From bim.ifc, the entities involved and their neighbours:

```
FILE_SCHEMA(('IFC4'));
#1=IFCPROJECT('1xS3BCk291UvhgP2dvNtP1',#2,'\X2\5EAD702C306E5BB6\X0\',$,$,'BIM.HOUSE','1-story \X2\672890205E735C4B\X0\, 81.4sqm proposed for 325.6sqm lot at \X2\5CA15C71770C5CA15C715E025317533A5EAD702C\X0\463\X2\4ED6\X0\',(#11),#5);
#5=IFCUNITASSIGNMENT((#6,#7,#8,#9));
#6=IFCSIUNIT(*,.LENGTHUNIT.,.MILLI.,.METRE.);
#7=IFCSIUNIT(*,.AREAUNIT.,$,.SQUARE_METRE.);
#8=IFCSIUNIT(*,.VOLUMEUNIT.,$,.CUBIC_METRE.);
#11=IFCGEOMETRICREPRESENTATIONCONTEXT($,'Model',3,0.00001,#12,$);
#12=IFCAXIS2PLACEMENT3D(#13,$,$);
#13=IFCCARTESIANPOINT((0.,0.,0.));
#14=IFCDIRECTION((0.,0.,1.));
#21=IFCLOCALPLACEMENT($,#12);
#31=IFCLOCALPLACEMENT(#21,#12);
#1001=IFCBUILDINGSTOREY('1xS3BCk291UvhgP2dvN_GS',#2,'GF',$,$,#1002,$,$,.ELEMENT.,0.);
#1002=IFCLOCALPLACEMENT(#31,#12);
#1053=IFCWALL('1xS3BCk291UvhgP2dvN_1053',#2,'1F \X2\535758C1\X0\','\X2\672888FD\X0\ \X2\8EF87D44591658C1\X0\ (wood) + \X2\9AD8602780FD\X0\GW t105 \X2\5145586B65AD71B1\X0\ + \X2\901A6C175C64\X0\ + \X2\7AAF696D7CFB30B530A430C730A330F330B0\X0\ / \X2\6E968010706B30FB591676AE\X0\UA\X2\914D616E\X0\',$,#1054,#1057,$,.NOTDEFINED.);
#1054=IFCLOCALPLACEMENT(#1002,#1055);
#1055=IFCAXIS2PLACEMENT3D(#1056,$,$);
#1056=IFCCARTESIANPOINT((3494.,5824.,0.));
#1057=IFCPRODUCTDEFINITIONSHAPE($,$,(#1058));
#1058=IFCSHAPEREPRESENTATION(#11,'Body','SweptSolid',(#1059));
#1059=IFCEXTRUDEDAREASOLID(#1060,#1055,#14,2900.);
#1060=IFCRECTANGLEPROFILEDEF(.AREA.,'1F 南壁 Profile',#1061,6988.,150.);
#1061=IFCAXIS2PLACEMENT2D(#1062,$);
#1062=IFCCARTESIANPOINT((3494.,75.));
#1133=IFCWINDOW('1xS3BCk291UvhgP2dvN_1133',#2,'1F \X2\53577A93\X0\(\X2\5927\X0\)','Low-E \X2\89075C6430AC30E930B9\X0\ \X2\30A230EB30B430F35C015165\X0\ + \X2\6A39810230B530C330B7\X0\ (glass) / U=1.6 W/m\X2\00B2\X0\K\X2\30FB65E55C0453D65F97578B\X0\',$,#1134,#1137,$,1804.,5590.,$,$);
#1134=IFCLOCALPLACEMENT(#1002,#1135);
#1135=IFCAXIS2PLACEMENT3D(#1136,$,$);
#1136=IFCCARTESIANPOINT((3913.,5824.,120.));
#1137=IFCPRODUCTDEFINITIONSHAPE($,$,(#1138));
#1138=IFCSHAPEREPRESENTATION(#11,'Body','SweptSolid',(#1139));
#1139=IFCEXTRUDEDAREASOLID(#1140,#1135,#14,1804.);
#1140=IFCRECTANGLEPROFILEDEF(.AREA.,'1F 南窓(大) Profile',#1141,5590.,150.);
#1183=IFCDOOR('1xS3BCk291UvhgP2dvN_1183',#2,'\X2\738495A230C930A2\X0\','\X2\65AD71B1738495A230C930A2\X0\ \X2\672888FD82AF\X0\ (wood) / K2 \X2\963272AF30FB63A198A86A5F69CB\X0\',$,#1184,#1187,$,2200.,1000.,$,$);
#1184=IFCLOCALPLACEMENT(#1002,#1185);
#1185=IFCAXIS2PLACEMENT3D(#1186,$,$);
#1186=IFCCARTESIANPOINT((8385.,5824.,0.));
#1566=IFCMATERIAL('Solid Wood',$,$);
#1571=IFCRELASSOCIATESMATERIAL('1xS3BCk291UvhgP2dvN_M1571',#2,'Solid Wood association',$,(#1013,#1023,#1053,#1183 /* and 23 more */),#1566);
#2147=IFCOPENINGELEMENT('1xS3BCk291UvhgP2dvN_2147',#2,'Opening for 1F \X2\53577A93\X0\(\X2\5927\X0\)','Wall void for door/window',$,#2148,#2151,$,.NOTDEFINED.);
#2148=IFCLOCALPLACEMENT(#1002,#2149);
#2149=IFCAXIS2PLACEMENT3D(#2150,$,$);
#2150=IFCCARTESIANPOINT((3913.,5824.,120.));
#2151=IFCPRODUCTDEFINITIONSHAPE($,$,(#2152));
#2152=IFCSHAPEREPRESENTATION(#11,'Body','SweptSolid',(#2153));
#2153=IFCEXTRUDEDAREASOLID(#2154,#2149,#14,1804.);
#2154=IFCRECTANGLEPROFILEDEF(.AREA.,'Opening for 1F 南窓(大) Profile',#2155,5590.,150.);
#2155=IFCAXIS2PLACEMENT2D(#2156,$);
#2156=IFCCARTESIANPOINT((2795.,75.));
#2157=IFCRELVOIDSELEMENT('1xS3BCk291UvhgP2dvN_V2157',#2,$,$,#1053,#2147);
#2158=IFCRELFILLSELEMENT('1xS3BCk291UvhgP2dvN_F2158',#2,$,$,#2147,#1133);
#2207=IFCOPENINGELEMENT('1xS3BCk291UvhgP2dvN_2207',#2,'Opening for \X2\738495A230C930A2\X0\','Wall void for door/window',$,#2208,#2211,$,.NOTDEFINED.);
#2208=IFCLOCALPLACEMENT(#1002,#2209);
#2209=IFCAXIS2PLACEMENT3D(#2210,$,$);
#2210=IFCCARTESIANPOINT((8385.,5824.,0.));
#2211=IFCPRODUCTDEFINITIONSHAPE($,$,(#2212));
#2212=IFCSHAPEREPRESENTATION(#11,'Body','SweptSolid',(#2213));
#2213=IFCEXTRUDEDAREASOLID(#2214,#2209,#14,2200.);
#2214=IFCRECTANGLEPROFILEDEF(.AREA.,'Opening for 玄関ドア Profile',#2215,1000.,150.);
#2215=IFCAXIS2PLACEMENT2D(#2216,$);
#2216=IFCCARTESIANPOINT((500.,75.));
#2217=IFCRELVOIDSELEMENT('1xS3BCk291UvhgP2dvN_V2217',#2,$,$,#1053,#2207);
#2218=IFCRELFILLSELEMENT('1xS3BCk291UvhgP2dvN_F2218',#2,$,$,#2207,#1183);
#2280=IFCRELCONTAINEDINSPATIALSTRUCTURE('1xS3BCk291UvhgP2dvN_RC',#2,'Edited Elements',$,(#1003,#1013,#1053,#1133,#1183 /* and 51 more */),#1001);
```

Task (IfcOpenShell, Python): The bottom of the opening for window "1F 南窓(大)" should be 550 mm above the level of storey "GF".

```python
import numpy as np
import ifcopenshell
import ifcopenshell.api.geometry
import ifcopenshell.geom
import ifcopenshell.util.element
import ifcopenshell.util.placement
import ifcopenshell.util.shape
import ifcopenshell.util.unit

model = ifcopenshell.open("bim.ifc")
unit_scale = ifcopenshell.util.unit.calculate_unit_scale(model)

window = model.by_guid("1xS3BCk291UvhgP2dvN_1133")
opening = window.FillsVoids[0].RelatingOpeningElement
storey = ifcopenshell.util.element.get_container(window, ifc_class="IfcBuildingStorey")
level = ifcopenshell.util.placement.get_local_placement(storey.ObjectPlacement)[2, 3]

# The opening's origin need not be at the sill, so measure its lowest point.
shape = ifcopenshell.geom.create_shape(ifcopenshell.geom.settings(), opening)
bottom = ifcopenshell.util.shape.get_shape_bottom_elevation(shape, shape.geometry) / unit_scale
dz = level + 550.0 - bottom

shift = np.array([0.0, 0.0, dz])
# The window is not placed relative to its opening, so move both.
for product in (opening, window):
    matrix = ifcopenshell.util.placement.get_local_placement(product.ObjectPlacement)
    matrix[:3, 3] += shift
    ifcopenshell.api.geometry.edit_object_placement(model, product=product, matrix=matrix, is_si=False)

print(f"moved by {dz * unit_scale:+.3f} m")

model.write("bim_v2.ifc")
```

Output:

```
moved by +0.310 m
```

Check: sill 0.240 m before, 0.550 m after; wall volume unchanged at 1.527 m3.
